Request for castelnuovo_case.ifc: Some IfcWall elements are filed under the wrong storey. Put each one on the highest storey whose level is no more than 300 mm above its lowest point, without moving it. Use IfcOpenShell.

First a look at what the model holds.

```python
import ifcopenshell
import ifcopenshell.util.element
import ifcopenshell.util.placement

model = ifcopenshell.open("castelnuovo_case.ifc")
print(model.schema)
for storey in model.by_type("IfcBuildingStorey"):
    level = ifcopenshell.util.placement.get_storey_elevation(storey)
    count = sum(e.is_a("IfcWall") for e in ifcopenshell.util.element.get_contained(storey))
    print(storey.id(), storey.Name, round(level, 3), count, sep=" | ")
```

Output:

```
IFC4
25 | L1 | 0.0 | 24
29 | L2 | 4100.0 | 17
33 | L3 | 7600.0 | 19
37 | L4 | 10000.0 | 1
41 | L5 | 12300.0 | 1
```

```python
import ifcopenshell
import ifcopenshell.api.spatial
import ifcopenshell.geom
import ifcopenshell.util.element
import ifcopenshell.util.placement
import ifcopenshell.util.shape
import ifcopenshell.util.unit

model = ifcopenshell.open("castelnuovo_case.ifc")
unit_scale = ifcopenshell.util.unit.calculate_unit_scale(model)
settings = ifcopenshell.geom.settings()

levels = sorted(
    ((ifcopenshell.util.placement.get_storey_elevation(s) * unit_scale, s) for s in model.by_type("IfcBuildingStorey")),
    key=lambda pair: pair[0],
)

for e in model.by_type("IfcWall"):
    current = e.ContainedInStructure[0].RelatingStructure if e.ContainedInStructure else None
    if current is None or not current.is_a("IfcBuildingStorey"):
        continue
    shape = ifcopenshell.geom.create_shape(settings, e)
    bottom = ifcopenshell.util.shape.get_shape_bottom_elevation(shape, shape.geometry)
    below = [s for level, s in levels if level <= bottom + 0.3]
    storey = below[-1] if below else levels[0][1]
    if storey != current:
        # assign_container keeps the world position.
        ifcopenshell.api.spatial.assign_container(model, products=[e], relating_structure=storey)
        print(e.id(), current.Name, "->", storey.Name)

model.write("castelnuovo_case-out.ifc")
```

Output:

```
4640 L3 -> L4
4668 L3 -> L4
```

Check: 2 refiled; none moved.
